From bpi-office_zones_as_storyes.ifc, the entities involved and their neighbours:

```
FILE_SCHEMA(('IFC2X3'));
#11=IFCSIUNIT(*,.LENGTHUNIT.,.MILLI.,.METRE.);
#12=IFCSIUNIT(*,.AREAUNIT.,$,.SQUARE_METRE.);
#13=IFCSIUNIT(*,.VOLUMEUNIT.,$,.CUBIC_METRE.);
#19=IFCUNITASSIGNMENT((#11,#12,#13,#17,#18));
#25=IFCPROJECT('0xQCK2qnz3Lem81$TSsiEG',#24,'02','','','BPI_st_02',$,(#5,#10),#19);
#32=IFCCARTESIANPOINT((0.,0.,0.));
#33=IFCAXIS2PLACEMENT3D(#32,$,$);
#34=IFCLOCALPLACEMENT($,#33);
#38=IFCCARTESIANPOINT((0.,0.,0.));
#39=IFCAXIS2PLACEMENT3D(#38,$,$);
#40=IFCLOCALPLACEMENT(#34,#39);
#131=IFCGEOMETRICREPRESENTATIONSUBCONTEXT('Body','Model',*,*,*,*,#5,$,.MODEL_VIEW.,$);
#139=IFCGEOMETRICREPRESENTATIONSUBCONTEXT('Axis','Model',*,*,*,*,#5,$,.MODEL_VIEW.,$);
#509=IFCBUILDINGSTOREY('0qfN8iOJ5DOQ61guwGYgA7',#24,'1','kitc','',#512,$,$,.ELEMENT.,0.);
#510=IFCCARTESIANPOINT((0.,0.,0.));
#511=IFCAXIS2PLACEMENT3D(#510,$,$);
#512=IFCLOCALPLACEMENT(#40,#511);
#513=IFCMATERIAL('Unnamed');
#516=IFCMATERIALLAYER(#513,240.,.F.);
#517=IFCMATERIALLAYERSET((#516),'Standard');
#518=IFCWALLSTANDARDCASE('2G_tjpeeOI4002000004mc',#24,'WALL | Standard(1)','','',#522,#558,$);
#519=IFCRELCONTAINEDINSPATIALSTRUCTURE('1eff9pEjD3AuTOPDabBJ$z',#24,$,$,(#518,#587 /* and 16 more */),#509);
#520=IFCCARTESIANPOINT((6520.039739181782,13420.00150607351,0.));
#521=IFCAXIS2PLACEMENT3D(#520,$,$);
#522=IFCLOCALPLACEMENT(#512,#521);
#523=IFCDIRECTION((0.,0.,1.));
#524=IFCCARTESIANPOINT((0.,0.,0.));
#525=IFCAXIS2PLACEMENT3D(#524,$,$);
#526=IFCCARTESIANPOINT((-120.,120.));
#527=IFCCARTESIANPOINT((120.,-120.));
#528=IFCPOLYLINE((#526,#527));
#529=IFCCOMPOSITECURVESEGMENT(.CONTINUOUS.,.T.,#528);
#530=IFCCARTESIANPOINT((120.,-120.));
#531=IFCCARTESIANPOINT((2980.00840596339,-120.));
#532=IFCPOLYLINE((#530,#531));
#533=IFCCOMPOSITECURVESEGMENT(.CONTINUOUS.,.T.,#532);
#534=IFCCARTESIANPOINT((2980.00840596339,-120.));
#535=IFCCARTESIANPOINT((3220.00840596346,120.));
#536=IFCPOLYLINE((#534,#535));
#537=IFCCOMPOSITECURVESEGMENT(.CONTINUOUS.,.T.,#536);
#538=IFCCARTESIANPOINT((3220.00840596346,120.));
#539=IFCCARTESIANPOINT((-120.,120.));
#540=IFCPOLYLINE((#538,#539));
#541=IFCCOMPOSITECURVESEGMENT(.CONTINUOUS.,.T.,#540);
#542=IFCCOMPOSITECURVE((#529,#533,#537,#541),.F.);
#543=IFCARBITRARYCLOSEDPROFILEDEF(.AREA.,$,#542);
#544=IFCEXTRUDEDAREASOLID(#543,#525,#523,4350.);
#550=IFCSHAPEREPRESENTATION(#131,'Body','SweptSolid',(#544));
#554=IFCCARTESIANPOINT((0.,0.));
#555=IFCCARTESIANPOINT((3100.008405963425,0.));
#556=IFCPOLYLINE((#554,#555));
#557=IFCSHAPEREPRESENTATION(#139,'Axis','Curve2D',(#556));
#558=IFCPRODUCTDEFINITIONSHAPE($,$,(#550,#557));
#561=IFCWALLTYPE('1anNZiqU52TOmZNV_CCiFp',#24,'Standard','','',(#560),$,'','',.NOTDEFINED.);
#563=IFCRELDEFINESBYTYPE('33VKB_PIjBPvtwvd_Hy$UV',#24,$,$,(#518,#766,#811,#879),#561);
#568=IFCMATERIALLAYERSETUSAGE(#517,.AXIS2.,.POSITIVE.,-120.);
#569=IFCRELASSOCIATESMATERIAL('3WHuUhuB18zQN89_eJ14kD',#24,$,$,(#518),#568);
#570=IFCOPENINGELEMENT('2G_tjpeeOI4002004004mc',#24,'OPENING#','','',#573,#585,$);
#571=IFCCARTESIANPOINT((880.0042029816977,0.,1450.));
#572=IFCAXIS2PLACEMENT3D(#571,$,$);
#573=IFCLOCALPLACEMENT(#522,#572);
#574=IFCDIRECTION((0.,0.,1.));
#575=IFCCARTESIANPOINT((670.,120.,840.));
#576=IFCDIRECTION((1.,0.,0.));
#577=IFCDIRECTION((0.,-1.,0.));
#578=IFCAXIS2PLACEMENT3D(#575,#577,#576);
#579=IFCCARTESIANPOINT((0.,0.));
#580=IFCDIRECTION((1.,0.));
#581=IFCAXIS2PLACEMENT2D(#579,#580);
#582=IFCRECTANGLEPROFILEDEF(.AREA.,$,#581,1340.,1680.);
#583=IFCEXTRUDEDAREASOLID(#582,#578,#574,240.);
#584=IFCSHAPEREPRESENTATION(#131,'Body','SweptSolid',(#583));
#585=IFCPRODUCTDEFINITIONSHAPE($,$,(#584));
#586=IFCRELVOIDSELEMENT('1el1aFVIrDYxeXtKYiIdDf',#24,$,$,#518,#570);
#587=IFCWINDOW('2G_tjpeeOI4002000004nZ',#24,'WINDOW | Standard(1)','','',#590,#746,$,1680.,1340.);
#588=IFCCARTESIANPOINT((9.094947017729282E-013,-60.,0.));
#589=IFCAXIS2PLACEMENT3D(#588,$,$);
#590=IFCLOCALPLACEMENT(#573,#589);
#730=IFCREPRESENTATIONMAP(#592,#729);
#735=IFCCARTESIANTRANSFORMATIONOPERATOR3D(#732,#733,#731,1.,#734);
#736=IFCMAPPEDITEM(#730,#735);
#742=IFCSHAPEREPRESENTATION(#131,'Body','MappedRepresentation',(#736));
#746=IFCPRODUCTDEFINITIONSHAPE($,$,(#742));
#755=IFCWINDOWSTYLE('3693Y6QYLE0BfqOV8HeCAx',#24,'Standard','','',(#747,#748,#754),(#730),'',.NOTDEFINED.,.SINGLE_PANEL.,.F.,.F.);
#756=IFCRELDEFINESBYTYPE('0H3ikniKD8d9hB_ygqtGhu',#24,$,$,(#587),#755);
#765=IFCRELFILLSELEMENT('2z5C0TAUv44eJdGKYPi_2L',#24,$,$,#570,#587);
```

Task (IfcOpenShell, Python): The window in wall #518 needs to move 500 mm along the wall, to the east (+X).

```python
import ifcopenshell
import ifcopenshell.api.geometry
import ifcopenshell.util.placement

model = ifcopenshell.open("bpi-office_zones_as_storyes.ifc")

window = model.by_id(587)
opening = window.FillsVoids[0].RelatingOpeningElement
wall = opening.VoidsElements[0].RelatingBuildingElement

wall_matrix = ifcopenshell.util.placement.get_local_placement(wall.ObjectPlacement)
shift = wall_matrix[:3, 0] * 500.0
before = ifcopenshell.util.placement.get_local_placement(window.ObjectPlacement)[:3, 3].copy()

# The window is placed relative to its opening, so it follows when the opening moves.
matrix = ifcopenshell.util.placement.get_local_placement(opening.ObjectPlacement)
matrix[:3, 3] += shift
ifcopenshell.api.geometry.edit_object_placement(
    model, product=opening, matrix=matrix, is_si=False, should_transform_children=True
)

after = ifcopenshell.util.placement.get_local_placement(window.ObjectPlacement)[:3, 3]
print("window moved by", (after - before).round(3) + 0.0)

model.write("bpi-office_zones_as_storyes_updated.ifc")
```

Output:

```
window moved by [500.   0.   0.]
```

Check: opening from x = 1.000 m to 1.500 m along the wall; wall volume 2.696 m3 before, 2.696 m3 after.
